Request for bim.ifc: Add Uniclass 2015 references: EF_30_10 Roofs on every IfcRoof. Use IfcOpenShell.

First a look at what the model holds.

```python
import ifcopenshell

model = ifcopenshell.open("bim.ifc")
print(model.schema)
print("classifications:", [c.Name for c in model.by_type("IfcClassification")])
for ifc_class in ("IfcDoor", "IfcRoof", "IfcStair", "IfcWall", "IfcWindow"):
    print(ifc_class, len(model.by_type(ifc_class)))
```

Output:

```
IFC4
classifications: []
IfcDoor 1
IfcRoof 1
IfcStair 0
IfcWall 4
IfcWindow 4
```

```python
import ifcopenshell
import ifcopenshell.api.classification

model = ifcopenshell.open("bim.ifc")

system = ifcopenshell.api.classification.add_classification(model, classification="Uniclass 2015")

codes = {
    "IfcRoof": ("EF_30_10", "Roofs"),
}
for ifc_class, (code, name) in codes.items():
    products = model.by_type(ifc_class)
    ifcopenshell.api.classification.add_reference(
        model, products=products, classification=system, identification=code, name=name
    )
    print(code, len(products))

model.write("bim_updated.ifc")
```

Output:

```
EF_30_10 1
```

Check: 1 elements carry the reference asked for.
